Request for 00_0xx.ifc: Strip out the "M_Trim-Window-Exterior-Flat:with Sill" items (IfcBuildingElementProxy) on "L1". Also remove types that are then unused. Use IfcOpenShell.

First a look at what the model holds.

```python
import ifcopenshell
import ifcopenshell.util.element

model = ifcopenshell.open("00_0xx.ifc")
print(model.schema)
storey = next(s for s in model.by_type("IfcBuildingStorey") if s.Name == "L1")
proxies = [e for e in ifcopenshell.util.element.get_decomposition(storey) if e.is_a("IfcBuildingElementProxy")]
seen = {}
for e in proxies:
    element_type = ifcopenshell.util.element.get_type(e)
    name = element_type.Name if element_type not in (None, e) else None
    seen[name] = seen.get(name, 0) + 1
for name, count in sorted(seen.items(), key=str):
    print(count, "x", name)
```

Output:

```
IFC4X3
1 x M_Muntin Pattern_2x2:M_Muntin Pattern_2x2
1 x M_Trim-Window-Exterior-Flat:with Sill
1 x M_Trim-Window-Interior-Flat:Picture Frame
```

```python
import ifcopenshell
import ifcopenshell.api.root
import ifcopenshell.util.element

model = ifcopenshell.open("00_0xx.ifc")

storey = next(s for s in model.by_type("IfcBuildingStorey") if s.Name == "L1")
proxies = [e for e in ifcopenshell.util.element.get_decomposition(storey) if e.is_a("IfcBuildingElementProxy")]
targets = [e for e in proxies if (t := ifcopenshell.util.element.get_type(e)) not in (None, e) and t.Name == "M_Trim-Window-Exterior-Flat:with Sill"]
types = {ifcopenshell.util.element.get_type(e) for e in targets} - {None, *targets}

for e in targets:
    ifcopenshell.api.root.remove_product(model, product=e)
print(len(targets), "removed")

unused = [t for t in types if not ifcopenshell.util.element.get_types(t)]
for t in unused:
    ifcopenshell.api.root.remove_product(model, product=t)
print(len(unused), "unused types removed")

model.write("00_0xx_edited.ifc")
```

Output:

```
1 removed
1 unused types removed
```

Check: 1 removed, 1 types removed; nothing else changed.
